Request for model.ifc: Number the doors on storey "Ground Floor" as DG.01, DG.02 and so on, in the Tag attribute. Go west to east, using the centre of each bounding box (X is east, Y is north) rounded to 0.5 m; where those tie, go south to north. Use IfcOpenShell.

First a look at what the model holds.

```python
import ifcopenshell
import ifcopenshell.util.element
import ifcopenshell.util.placement

model = ifcopenshell.open("model.ifc")
print(model.schema)
storey = next(s for s in model.by_type("IfcBuildingStorey") if s.Name == "Ground Floor")
doors = [e for e in ifcopenshell.util.element.get_decomposition(storey) if e.is_a("IfcDoor")]
for e in sorted(doors, key=lambda e: e.id()):
    origin = ifcopenshell.util.placement.get_local_placement(e.ObjectPlacement)[:3, 3]
    print(e.id(), e.Tag, e.Name, origin.round(2) + 0.0, sep=" | ")
```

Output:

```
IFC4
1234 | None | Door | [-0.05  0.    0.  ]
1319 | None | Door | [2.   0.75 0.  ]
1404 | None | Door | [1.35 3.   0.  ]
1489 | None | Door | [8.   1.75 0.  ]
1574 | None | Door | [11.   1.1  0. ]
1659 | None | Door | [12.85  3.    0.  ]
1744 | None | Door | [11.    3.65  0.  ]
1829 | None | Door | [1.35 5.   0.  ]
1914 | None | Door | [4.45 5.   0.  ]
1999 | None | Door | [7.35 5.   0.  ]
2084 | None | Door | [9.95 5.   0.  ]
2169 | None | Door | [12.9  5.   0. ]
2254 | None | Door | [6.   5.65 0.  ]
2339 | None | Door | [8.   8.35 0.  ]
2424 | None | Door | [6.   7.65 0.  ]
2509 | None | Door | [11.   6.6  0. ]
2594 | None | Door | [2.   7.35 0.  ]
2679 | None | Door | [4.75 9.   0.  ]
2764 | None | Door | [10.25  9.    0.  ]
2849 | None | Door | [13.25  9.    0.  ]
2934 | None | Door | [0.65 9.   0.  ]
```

```python
import ifcopenshell
import ifcopenshell.geom
import ifcopenshell.util.element
import ifcopenshell.util.shape

model = ifcopenshell.open("model.ifc")
settings = ifcopenshell.geom.settings()
settings.set("use-world-coords", True)


def centre(element):
    shape = ifcopenshell.geom.create_shape(settings, element)
    return ifcopenshell.util.shape.get_bbox_centroid(shape.geometry)


storey = next(s for s in model.by_type("IfcBuildingStorey") if s.Name == "Ground Floor")
doors = [e for e in ifcopenshell.util.element.get_decomposition(storey) if e.is_a("IfcDoor")]

# Insertion points can sit at a corner or the storey origin, so sort by the geometry (in metres).
centres = {e: centre(e) for e in doors}
doors.sort(key=lambda e: (round(centres[e][0] / 0.5), centres[e][1]))

for i, e in enumerate(doors, start=1):
    number = f"DG.{i:02d}"
    e.Tag = number
    print(e.id(), number)

model.write("model_updated.ifc")
```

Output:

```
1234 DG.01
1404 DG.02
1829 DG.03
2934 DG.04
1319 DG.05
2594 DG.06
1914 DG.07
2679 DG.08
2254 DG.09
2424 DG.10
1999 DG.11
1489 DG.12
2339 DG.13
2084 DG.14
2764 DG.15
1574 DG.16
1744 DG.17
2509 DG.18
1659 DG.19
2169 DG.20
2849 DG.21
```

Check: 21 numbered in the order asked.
